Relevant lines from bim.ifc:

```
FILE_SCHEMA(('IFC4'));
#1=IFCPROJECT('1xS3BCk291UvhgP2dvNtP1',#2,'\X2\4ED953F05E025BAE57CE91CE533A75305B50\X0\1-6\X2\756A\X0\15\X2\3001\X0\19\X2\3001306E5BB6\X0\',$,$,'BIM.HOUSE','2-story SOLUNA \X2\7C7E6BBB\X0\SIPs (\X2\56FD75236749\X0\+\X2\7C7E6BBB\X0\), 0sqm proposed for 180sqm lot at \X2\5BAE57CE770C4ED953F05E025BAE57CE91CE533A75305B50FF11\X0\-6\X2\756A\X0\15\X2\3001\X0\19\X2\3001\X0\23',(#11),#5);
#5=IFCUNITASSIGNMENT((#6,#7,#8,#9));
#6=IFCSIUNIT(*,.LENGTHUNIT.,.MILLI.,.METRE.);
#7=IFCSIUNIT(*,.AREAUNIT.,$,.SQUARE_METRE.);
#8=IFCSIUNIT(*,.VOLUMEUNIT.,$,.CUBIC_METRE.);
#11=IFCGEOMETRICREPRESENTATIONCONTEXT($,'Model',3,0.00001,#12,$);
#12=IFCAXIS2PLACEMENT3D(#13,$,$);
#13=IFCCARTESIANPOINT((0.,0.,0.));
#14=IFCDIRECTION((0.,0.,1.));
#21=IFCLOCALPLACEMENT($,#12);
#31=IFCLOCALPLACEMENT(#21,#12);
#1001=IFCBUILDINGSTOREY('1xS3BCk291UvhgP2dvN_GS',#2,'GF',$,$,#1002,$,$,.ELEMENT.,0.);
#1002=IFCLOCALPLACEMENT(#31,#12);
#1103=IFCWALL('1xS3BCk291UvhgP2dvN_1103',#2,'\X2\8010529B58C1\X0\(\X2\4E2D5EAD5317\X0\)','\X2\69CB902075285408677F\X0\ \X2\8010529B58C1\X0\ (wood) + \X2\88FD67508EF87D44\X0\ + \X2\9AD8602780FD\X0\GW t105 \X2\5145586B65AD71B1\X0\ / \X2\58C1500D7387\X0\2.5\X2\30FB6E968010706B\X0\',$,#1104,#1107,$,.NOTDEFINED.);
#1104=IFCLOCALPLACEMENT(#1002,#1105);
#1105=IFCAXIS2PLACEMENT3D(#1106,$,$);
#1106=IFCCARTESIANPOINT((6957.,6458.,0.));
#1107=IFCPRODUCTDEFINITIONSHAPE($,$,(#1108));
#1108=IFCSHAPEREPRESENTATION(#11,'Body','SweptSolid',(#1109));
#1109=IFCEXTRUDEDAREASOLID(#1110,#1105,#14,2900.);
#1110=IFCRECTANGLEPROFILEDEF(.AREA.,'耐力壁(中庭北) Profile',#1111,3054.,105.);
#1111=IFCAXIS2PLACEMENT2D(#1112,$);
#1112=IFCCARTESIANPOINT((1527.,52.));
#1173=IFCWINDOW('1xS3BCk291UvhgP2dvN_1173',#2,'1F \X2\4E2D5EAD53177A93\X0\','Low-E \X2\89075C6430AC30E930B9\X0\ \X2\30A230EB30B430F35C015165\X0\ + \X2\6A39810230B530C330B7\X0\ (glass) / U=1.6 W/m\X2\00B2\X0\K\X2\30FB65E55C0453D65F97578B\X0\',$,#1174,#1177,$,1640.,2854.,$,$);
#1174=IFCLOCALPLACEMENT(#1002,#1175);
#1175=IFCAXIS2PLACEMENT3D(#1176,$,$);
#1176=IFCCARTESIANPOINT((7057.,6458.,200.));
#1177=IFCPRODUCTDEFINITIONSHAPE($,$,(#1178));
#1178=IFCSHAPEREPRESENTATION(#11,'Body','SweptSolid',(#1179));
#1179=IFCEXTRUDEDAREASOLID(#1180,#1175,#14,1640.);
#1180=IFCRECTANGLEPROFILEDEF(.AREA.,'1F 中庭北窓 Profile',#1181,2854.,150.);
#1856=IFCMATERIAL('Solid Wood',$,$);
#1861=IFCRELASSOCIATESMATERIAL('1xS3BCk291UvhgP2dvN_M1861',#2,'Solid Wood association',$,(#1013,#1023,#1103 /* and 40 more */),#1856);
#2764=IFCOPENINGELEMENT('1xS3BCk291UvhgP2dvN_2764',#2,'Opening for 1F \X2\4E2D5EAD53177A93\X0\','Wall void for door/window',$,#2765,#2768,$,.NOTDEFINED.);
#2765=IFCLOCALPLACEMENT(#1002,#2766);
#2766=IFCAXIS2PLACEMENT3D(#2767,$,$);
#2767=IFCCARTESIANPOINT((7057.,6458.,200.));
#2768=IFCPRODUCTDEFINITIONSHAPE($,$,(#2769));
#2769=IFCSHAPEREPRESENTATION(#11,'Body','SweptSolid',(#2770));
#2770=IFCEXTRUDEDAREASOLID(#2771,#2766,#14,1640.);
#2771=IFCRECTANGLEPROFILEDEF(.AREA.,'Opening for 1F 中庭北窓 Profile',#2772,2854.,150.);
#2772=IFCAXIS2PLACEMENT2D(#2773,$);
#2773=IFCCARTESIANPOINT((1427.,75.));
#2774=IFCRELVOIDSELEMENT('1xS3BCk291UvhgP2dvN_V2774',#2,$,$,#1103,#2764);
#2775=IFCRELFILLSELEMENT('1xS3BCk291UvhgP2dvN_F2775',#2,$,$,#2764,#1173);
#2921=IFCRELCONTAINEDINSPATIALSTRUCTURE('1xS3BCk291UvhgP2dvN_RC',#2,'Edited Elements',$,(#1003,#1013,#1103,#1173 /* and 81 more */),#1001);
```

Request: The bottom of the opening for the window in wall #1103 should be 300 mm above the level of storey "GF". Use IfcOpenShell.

```python
import numpy as np
import ifcopenshell
import ifcopenshell.api.geometry
import ifcopenshell.geom
import ifcopenshell.util.element
import ifcopenshell.util.placement
import ifcopenshell.util.shape
import ifcopenshell.util.unit

model = ifcopenshell.open("bim.ifc")
unit_scale = ifcopenshell.util.unit.calculate_unit_scale(model)

window = model.by_guid("1xS3BCk291UvhgP2dvN_1173")
opening = window.FillsVoids[0].RelatingOpeningElement
storey = ifcopenshell.util.element.get_container(window, ifc_class="IfcBuildingStorey")
level = ifcopenshell.util.placement.get_local_placement(storey.ObjectPlacement)[2, 3]

# The opening's origin need not be at the sill, so measure its lowest point.
shape = ifcopenshell.geom.create_shape(ifcopenshell.geom.settings(), opening)
bottom = ifcopenshell.util.shape.get_shape_bottom_elevation(shape, shape.geometry) / unit_scale
dz = level + 0.3 / unit_scale - bottom

shift = np.array([0.0, 0.0, dz])
# The window is not placed relative to its opening, so move both.
for product in (opening, window):
    matrix = ifcopenshell.util.placement.get_local_placement(product.ObjectPlacement)
    matrix[:3, 3] += shift
    ifcopenshell.api.geometry.edit_object_placement(model, product=product, matrix=matrix, is_si=False)

print(f"moved by {dz * unit_scale:+.3f} m")

model.write("bim_edited.ifc")
```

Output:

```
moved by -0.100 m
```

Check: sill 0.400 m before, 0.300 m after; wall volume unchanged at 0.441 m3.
